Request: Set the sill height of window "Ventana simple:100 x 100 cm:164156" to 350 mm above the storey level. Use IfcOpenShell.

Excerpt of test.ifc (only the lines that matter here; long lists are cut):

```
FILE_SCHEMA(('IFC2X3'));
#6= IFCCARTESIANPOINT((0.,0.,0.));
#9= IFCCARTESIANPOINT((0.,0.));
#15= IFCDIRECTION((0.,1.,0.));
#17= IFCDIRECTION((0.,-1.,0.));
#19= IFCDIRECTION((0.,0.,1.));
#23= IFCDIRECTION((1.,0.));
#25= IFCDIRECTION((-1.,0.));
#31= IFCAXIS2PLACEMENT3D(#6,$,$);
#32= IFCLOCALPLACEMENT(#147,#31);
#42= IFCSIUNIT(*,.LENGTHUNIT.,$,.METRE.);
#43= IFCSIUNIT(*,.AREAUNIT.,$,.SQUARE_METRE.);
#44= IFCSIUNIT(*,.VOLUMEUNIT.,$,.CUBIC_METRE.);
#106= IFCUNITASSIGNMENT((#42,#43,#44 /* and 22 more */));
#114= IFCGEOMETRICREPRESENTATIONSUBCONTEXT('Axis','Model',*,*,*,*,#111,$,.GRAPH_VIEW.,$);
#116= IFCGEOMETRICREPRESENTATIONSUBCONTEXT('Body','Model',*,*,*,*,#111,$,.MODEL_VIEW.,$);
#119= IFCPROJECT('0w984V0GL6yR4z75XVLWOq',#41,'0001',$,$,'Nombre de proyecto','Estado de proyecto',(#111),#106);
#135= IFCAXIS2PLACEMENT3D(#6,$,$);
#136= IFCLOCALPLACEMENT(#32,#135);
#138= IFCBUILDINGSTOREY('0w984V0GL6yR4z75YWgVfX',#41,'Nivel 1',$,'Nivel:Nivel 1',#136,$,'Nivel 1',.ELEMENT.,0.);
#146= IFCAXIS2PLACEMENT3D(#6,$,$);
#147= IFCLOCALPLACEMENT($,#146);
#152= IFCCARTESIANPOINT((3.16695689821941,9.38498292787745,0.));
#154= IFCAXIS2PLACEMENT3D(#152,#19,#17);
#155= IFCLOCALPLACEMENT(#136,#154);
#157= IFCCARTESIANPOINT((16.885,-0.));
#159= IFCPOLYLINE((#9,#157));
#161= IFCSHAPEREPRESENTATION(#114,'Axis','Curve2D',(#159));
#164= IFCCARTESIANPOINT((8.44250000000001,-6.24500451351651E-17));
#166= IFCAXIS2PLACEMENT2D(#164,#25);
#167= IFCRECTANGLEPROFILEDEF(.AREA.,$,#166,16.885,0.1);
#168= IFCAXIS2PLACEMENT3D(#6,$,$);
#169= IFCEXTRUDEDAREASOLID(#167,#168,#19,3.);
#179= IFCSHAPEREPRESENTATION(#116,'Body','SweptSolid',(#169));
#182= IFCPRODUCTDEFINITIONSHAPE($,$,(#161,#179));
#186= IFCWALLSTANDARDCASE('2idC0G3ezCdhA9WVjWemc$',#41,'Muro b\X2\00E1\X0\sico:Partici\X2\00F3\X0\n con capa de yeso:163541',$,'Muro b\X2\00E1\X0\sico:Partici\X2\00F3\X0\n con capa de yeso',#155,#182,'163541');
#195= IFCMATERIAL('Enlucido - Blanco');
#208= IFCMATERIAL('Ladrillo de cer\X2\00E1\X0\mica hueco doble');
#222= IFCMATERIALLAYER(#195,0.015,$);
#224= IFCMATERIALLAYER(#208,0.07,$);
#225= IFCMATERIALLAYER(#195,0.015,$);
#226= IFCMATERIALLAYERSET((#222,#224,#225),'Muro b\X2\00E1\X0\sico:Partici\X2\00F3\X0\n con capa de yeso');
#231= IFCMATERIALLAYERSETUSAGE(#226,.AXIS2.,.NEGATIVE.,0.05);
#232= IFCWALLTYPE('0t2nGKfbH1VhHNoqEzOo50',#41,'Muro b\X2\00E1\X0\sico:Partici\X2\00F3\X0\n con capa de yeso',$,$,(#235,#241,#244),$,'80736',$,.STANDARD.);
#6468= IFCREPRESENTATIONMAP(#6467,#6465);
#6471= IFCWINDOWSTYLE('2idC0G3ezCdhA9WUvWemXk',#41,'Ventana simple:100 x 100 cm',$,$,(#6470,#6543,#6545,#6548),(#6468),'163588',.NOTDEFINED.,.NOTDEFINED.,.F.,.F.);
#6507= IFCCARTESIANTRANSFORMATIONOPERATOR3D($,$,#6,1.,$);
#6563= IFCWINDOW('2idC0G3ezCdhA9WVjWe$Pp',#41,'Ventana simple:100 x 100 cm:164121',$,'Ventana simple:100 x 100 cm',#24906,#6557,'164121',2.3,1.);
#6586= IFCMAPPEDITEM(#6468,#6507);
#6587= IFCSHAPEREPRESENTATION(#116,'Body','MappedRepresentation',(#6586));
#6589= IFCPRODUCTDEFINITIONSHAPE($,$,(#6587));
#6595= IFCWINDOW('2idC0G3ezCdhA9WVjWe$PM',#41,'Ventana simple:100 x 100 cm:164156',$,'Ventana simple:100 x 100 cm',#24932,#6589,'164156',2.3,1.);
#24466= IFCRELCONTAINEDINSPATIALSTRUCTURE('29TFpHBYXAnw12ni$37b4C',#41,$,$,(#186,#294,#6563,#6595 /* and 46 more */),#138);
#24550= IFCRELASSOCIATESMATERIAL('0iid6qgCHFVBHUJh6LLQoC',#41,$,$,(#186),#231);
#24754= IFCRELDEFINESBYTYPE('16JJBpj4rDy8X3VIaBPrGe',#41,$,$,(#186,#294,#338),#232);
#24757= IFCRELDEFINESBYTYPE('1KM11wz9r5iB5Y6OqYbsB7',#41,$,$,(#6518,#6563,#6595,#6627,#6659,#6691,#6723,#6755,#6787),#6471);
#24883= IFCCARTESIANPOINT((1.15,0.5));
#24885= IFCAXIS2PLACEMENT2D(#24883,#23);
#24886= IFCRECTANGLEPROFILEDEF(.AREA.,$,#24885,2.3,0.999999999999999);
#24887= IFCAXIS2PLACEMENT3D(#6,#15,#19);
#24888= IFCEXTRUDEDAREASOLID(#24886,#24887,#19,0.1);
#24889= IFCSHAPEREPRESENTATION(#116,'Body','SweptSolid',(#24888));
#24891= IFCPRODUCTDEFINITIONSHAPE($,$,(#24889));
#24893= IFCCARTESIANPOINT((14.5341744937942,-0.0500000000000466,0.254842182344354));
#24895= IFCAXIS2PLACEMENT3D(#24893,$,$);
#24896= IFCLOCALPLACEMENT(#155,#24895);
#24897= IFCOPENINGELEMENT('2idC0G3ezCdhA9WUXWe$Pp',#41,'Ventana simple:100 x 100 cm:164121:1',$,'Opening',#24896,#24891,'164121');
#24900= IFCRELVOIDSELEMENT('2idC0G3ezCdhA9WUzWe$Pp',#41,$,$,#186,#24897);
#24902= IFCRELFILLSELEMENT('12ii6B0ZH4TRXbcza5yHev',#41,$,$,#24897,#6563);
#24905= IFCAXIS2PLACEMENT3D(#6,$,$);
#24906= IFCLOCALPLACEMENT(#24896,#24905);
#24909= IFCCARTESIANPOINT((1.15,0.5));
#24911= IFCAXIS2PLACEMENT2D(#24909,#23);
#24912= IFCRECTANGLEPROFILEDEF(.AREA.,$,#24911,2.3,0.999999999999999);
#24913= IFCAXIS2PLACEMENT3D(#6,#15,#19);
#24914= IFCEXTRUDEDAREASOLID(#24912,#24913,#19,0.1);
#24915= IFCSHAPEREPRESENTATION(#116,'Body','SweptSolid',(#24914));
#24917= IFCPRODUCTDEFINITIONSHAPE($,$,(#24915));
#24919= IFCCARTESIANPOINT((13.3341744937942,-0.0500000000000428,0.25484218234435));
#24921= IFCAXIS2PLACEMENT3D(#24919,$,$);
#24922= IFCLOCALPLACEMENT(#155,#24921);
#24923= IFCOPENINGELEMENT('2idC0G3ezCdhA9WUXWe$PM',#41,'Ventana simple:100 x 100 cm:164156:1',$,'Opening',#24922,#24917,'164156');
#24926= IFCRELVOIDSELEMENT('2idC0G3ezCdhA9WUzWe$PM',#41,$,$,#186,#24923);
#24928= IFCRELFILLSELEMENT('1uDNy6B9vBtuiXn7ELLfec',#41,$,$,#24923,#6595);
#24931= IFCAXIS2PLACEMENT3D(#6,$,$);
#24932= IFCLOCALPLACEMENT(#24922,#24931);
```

```python
import numpy as np
import ifcopenshell
import ifcopenshell.api.geometry
import ifcopenshell.geom
import ifcopenshell.util.element
import ifcopenshell.util.placement
import ifcopenshell.util.shape
import ifcopenshell.util.unit

model = ifcopenshell.open("test.ifc")
unit_scale = ifcopenshell.util.unit.calculate_unit_scale(model)

window = model.by_guid("2idC0G3ezCdhA9WVjWe$PM")
opening = window.FillsVoids[0].RelatingOpeningElement
storey = ifcopenshell.util.element.get_container(window, ifc_class="IfcBuildingStorey")
level = ifcopenshell.util.placement.get_local_placement(storey.ObjectPlacement)[2, 3]

# The opening's origin need not be at the sill, so measure its lowest point.
shape = ifcopenshell.geom.create_shape(ifcopenshell.geom.settings(), opening)
bottom = ifcopenshell.util.shape.get_shape_bottom_elevation(shape, shape.geometry) / unit_scale
dz = level + 0.35 / unit_scale - bottom

shift = np.array([0.0, 0.0, dz])
# The window is placed relative to its opening, so it follows when the opening moves.
matrix = ifcopenshell.util.placement.get_local_placement(opening.ObjectPlacement)
matrix[:3, 3] += shift
ifcopenshell.api.geometry.edit_object_placement(
    model, product=opening, matrix=matrix, is_si=False, should_transform_children=True
)

print(f"moved by {dz * unit_scale:+.3f} m")

model.write("test_updated.ifc")
```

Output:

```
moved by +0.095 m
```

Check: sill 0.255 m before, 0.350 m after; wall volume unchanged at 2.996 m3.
